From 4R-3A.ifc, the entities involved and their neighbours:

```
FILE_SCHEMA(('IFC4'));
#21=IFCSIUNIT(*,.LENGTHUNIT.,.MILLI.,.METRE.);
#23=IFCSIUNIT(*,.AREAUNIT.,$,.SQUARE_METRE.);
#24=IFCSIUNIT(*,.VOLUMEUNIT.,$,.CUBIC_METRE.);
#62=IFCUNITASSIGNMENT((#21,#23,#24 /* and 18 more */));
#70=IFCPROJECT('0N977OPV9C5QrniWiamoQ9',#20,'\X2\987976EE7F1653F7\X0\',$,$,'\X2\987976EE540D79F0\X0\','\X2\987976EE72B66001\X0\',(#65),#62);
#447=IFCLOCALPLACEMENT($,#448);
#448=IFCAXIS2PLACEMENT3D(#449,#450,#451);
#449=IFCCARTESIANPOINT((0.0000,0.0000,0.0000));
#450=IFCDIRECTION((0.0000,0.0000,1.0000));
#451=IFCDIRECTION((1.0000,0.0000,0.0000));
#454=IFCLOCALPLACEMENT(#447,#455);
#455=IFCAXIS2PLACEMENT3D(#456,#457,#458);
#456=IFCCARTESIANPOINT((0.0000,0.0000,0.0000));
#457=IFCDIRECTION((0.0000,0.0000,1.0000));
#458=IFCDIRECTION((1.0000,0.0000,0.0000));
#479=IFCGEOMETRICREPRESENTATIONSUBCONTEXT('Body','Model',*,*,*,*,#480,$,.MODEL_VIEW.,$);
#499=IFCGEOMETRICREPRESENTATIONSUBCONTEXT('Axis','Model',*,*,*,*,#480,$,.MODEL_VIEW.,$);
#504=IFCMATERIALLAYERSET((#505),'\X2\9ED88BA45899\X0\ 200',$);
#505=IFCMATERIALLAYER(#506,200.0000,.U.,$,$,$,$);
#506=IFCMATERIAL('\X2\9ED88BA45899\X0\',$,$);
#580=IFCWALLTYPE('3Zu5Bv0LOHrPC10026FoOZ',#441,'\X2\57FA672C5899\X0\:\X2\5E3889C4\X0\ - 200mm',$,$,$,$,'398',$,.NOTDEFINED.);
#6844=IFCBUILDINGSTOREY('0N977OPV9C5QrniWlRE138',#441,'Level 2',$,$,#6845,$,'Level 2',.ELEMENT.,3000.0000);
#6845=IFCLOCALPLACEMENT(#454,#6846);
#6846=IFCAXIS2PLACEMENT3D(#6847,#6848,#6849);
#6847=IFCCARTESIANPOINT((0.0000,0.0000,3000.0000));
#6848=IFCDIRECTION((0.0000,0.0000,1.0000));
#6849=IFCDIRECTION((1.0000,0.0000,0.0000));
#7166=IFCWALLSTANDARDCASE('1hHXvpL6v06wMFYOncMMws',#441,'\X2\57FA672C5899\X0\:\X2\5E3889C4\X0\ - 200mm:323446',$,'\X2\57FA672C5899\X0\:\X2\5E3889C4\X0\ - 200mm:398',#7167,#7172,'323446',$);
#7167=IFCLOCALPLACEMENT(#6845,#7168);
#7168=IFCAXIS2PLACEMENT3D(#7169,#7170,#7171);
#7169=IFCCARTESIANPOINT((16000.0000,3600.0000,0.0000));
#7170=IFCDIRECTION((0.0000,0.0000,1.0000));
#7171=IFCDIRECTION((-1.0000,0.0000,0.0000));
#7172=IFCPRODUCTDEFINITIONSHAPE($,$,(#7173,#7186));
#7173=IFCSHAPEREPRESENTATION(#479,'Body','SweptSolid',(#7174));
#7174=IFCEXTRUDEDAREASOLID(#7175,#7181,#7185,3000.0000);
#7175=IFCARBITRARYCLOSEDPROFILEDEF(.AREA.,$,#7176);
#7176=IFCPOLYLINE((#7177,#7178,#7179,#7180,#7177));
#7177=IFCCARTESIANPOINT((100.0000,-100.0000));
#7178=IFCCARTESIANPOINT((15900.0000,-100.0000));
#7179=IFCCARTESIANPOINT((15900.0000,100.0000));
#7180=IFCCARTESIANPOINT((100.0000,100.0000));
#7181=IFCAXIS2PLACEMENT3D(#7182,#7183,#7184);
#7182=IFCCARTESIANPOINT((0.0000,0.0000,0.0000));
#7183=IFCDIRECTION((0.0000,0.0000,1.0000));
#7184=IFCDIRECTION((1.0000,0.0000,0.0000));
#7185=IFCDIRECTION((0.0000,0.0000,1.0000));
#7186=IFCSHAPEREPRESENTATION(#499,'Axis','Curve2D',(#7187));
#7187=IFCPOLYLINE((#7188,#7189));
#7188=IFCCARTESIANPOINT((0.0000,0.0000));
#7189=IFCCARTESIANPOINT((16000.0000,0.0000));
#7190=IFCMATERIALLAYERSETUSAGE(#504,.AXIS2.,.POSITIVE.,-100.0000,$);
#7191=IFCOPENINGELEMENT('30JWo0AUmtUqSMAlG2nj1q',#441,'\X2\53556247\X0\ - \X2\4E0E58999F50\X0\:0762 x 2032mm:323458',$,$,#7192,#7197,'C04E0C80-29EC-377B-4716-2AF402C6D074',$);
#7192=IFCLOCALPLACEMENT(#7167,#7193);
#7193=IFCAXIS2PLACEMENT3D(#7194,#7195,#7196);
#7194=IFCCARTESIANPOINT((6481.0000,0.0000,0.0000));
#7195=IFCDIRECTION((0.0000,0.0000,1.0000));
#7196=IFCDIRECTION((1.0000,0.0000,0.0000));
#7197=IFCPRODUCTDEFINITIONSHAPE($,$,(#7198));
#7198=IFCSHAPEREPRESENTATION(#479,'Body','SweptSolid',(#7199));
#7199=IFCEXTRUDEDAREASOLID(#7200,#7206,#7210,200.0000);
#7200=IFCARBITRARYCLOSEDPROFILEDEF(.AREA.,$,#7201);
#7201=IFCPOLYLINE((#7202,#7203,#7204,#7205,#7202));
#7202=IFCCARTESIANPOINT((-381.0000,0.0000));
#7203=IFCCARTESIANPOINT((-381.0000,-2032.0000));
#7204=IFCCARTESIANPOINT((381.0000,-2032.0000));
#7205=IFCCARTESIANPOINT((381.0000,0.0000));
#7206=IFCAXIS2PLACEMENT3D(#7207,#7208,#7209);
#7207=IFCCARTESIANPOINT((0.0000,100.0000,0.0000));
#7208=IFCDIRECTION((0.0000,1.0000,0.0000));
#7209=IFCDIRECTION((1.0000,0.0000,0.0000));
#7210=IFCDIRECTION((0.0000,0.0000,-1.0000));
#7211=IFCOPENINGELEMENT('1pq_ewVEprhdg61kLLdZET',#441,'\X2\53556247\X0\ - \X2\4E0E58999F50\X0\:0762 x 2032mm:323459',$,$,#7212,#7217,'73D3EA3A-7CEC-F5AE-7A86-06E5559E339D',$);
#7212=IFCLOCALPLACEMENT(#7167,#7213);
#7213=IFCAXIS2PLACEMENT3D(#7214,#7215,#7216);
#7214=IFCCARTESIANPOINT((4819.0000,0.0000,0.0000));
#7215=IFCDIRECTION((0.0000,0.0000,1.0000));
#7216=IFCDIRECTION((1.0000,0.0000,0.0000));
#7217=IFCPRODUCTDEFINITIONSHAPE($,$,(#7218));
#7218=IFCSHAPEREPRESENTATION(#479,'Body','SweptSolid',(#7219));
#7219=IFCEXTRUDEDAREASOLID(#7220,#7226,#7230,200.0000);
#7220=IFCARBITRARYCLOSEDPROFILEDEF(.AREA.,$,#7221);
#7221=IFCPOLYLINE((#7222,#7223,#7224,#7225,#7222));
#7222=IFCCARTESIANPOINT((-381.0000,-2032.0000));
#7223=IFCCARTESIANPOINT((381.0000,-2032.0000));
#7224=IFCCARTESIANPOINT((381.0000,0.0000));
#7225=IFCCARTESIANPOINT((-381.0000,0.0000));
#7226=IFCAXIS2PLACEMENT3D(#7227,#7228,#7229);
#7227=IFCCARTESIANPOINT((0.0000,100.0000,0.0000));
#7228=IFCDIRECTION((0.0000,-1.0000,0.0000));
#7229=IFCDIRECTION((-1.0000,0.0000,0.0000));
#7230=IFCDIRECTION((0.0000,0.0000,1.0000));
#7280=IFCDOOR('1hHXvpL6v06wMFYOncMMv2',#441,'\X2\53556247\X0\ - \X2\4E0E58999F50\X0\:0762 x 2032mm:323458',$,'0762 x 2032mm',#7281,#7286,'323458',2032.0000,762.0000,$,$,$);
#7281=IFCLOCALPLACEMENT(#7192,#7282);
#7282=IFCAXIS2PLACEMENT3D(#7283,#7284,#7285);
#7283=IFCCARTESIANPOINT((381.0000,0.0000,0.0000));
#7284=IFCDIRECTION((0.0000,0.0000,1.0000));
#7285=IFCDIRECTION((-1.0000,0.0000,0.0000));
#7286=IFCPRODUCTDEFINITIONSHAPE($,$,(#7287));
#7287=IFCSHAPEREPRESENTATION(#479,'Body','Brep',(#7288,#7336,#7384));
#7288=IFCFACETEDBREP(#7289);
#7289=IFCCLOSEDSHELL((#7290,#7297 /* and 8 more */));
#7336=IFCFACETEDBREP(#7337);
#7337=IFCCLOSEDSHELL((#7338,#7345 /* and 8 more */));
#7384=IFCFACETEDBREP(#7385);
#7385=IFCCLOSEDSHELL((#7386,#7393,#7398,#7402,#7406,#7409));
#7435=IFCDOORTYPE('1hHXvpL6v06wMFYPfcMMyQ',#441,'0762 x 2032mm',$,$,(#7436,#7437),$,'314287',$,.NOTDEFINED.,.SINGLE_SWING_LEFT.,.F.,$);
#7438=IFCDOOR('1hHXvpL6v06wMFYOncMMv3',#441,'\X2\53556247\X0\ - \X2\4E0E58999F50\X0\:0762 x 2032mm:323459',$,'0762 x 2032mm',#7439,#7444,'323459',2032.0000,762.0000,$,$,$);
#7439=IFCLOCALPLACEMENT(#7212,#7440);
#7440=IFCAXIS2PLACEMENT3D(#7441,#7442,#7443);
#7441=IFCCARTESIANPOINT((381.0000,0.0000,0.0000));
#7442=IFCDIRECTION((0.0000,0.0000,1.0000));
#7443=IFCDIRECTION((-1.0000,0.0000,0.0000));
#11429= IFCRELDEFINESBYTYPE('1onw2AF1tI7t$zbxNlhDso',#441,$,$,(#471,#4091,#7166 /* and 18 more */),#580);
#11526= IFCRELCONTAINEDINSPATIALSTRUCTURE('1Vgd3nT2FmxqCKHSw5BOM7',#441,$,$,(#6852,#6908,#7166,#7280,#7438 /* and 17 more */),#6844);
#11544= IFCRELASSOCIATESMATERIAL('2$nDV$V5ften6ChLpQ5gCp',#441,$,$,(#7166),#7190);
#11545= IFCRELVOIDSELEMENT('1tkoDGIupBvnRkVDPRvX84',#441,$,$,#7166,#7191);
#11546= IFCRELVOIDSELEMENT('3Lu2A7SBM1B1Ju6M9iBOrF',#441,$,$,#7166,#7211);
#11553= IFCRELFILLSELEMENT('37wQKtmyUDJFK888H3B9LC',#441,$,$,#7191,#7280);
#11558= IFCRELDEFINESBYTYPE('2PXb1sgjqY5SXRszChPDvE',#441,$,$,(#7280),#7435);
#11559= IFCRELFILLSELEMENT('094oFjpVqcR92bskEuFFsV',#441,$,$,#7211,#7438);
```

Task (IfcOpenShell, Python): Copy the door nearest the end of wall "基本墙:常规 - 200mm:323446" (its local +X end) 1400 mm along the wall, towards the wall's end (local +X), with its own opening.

```python
import ifcopenshell
import ifcopenshell.api.feature
import ifcopenshell.api.geometry
import ifcopenshell.api.root
import ifcopenshell.geom
import ifcopenshell.util.element
import ifcopenshell.util.placement
import ifcopenshell.util.shape
import ifcopenshell.util.unit

model = ifcopenshell.open("4R-3A.ifc")
unit_scale = ifcopenshell.util.unit.calculate_unit_scale(model)
settings = ifcopenshell.geom.settings()


def volume(element):
    """Net volume in cubic metres, openings subtracted."""
    shape = ifcopenshell.geom.create_shape(settings, element)
    return ifcopenshell.util.shape.get_volume(shape.geometry)


def reuse_history(source, copy):
    """copy_class also copies each property set's owner history, people and application; keep the originals."""
    for rel in copy.IsDefinedBy:
        if rel.is_a("IfcRelDefinesByProperties") and (history := rel.RelatingPropertyDefinition.OwnerHistory):
            rel.RelatingPropertyDefinition.OwnerHistory = source.OwnerHistory
            ifcopenshell.util.element.remove_deep2(model, history)


door = model.by_guid("1hHXvpL6v06wMFYOncMMv2")
opening = door.FillsVoids[0].RelatingOpeningElement
wall = opening.VoidsElements[0].RelatingBuildingElement
before = volume(wall)
shift = ifcopenshell.util.placement.get_local_placement(wall.ObjectPlacement)[:3, 0] * 1.4 / unit_scale

# copy_class copies the void relationship, type, container and properties, but no geometry.
new_opening = ifcopenshell.api.root.copy_class(model, product=opening)
new_opening.Representation = ifcopenshell.util.element.copy_deep(
    model, opening.Representation, exclude=["IfcGeometricRepresentationContext", "IfcRepresentationMap"]
)
new_opening.Name = "单扇 - 与墙齐:0762 x 2032mm"
new_opening.Tag = None
new_door = ifcopenshell.api.root.copy_class(model, product=door)
new_door.Representation = ifcopenshell.util.element.copy_deep(
    model, door.Representation, exclude=["IfcGeometricRepresentationContext", "IfcRepresentationMap"]
)
new_door.Name = "单扇 - 与墙齐:0762 x 2032mm"
new_door.Tag = None
reuse_history(door, new_door)
ifcopenshell.api.feature.add_filling(model, opening=new_opening, element=new_door)

for old, new in ((opening, new_opening), (door, new_door)):
    matrix = ifcopenshell.util.placement.get_local_placement(old.ObjectPlacement)
    matrix[:3, 3] += shift
    ifcopenshell.api.geometry.edit_object_placement(model, product=new, matrix=matrix, is_si=False)

after = volume(wall)

print(f"wall volume {before:.3f} -> {after:.3f} m3")

model.write("4R-3A_edited.ifc")
```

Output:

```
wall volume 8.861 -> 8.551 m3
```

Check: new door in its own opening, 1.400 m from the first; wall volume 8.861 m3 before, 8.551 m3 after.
